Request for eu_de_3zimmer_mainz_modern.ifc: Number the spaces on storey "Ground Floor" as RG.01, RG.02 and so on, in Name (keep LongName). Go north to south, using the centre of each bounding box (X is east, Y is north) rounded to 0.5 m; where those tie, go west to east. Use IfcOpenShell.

First a look at what the model holds.

```python
import ifcopenshell
import ifcopenshell.util.element
import ifcopenshell.util.placement

model = ifcopenshell.open("eu_de_3zimmer_mainz_modern.ifc")
print(model.schema)
storey = next(s for s in model.by_type("IfcBuildingStorey") if s.Name == "Ground Floor")
spaces = [e for e in ifcopenshell.util.element.get_decomposition(storey) if e.is_a("IfcSpace")]
for e in sorted(spaces, key=lambda e: e.id()):
    origin = ifcopenshell.util.placement.get_local_placement(e.ObjectPlacement)[:3, 3]
    print(e.id(), e.Name, e.LongName, origin.round(2) + 0.0, sep=" | ")
```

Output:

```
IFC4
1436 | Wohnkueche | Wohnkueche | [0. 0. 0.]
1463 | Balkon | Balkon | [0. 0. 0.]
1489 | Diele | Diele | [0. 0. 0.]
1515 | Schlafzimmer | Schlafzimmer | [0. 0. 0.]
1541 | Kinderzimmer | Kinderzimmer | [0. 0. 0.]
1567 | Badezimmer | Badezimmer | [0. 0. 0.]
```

```python
import ifcopenshell
import ifcopenshell.geom
import ifcopenshell.util.element
import ifcopenshell.util.shape

model = ifcopenshell.open("eu_de_3zimmer_mainz_modern.ifc")
settings = ifcopenshell.geom.settings()
settings.set("use-world-coords", True)


def centre(element):
    shape = ifcopenshell.geom.create_shape(settings, element)
    return ifcopenshell.util.shape.get_bbox_centroid(shape.geometry)


storey = next(s for s in model.by_type("IfcBuildingStorey") if s.Name == "Ground Floor")
spaces = [e for e in ifcopenshell.util.element.get_decomposition(storey) if e.is_a("IfcSpace")]

# Insertion points can sit at a corner or the storey origin, so sort by the geometry (in metres).
centres = {e: centre(e) for e in spaces}
spaces.sort(key=lambda e: (-round(centres[e][1] / 0.5), centres[e][0]))

for i, e in enumerate(spaces, start=1):
    number = f"RG.{i:02d}"
    e.Name = number
    print(e.id(), number)

model.write("eu_de_3zimmer_mainz_modern_v2.ifc")
```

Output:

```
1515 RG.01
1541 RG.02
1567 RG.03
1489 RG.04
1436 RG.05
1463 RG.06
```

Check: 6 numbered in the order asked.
